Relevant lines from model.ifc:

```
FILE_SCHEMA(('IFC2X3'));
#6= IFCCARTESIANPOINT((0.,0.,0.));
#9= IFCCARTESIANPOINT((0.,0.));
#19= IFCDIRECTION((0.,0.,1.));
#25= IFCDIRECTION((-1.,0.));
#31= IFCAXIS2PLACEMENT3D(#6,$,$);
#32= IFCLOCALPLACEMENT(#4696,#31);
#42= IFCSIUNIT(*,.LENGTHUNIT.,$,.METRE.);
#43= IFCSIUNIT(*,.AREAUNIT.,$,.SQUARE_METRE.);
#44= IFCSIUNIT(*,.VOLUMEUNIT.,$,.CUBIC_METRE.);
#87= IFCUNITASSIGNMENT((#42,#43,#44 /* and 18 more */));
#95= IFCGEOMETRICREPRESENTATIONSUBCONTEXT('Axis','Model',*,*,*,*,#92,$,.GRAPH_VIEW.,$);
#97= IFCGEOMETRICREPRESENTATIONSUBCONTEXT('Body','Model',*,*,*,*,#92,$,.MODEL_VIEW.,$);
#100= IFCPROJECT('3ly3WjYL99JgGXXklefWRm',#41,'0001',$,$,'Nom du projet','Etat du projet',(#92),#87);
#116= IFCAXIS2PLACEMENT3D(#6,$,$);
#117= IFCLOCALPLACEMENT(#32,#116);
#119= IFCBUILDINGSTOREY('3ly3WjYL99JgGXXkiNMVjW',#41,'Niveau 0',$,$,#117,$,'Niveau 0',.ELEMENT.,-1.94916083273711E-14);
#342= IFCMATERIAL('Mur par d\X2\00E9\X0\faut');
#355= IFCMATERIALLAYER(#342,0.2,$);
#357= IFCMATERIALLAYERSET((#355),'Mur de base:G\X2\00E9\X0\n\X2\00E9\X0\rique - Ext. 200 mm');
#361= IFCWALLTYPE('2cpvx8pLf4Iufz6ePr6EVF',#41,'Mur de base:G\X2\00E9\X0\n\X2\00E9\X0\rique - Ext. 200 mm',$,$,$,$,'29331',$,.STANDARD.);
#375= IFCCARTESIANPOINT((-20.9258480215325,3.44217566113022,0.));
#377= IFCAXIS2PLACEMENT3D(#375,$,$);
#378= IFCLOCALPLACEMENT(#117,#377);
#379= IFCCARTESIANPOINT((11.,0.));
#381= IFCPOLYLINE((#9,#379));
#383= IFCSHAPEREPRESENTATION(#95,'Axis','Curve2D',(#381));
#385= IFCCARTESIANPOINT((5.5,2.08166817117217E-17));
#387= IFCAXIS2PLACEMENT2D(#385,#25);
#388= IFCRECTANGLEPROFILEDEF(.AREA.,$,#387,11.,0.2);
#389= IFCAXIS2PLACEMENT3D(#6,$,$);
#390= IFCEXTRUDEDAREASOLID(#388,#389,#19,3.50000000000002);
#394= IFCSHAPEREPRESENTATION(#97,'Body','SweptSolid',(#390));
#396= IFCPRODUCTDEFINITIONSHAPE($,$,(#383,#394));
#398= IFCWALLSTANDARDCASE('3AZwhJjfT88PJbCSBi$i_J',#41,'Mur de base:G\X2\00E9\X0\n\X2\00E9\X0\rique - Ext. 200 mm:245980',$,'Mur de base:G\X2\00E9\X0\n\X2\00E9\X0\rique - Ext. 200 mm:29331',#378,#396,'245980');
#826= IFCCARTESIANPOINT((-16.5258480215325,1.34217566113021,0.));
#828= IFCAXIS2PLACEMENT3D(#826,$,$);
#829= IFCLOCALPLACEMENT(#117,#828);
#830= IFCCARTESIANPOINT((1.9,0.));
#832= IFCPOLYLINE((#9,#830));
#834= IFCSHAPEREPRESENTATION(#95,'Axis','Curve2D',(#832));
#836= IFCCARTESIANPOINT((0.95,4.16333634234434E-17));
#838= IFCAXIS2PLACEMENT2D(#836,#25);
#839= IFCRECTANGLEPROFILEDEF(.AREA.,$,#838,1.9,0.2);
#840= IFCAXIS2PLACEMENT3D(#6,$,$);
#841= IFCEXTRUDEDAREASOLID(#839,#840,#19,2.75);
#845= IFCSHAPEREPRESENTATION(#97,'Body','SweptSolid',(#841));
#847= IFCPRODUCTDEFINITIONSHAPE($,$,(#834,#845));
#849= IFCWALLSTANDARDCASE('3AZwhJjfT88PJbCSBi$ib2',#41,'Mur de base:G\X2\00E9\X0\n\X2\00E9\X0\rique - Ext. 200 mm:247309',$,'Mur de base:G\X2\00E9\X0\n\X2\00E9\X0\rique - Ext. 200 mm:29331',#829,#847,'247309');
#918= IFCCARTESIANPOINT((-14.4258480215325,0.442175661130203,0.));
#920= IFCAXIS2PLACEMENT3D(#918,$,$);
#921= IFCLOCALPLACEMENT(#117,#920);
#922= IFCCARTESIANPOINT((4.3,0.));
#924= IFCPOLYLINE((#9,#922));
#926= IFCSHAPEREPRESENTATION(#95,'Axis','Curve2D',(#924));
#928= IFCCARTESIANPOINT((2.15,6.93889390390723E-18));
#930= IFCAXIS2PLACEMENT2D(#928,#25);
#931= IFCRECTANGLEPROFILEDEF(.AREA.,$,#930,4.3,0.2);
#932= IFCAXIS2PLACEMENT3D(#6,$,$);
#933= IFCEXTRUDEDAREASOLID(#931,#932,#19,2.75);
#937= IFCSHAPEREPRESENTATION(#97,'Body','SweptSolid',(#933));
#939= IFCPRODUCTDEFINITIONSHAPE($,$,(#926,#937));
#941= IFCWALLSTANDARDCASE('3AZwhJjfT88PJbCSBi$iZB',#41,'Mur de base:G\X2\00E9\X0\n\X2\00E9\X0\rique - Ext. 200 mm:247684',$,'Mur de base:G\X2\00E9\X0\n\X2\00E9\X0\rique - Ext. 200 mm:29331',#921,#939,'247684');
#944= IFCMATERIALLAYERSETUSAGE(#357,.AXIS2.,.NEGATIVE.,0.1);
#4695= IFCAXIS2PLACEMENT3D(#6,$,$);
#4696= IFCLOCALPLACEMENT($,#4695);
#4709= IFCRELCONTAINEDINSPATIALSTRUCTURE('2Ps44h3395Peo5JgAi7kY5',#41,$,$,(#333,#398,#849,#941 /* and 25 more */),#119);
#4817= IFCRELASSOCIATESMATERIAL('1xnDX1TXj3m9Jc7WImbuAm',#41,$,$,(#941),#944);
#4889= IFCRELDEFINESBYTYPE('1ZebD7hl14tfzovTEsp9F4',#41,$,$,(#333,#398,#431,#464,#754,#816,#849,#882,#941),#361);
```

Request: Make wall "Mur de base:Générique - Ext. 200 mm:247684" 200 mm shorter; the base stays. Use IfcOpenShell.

```python
import ifcopenshell
import ifcopenshell.geom
import ifcopenshell.util.representation
import ifcopenshell.util.shape
import ifcopenshell.util.unit

model = ifcopenshell.open("model.ifc")
unit_scale = ifcopenshell.util.unit.calculate_unit_scale(model)
settings = ifcopenshell.geom.settings()


def volume(element):
    """Net volume in cubic metres, openings subtracted."""
    shape = ifcopenshell.geom.create_shape(settings, element)
    return ifcopenshell.util.shape.get_volume(shape.geometry)


wall = model.by_id(941)
before = volume(wall)

body = ifcopenshell.util.representation.get_representation(wall, "Model", "Body")
solid = body.Items[0]
old_height = solid.Depth
solid.Depth -= 0.2 / unit_scale
after = volume(wall)

print(f"height {old_height:g} -> {solid.Depth:g}, volume {before:.3f} -> {after:.3f} m3")

model.write("model-out.ifc")
```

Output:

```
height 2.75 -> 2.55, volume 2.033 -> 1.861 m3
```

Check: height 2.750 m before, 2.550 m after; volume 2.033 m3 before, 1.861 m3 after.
